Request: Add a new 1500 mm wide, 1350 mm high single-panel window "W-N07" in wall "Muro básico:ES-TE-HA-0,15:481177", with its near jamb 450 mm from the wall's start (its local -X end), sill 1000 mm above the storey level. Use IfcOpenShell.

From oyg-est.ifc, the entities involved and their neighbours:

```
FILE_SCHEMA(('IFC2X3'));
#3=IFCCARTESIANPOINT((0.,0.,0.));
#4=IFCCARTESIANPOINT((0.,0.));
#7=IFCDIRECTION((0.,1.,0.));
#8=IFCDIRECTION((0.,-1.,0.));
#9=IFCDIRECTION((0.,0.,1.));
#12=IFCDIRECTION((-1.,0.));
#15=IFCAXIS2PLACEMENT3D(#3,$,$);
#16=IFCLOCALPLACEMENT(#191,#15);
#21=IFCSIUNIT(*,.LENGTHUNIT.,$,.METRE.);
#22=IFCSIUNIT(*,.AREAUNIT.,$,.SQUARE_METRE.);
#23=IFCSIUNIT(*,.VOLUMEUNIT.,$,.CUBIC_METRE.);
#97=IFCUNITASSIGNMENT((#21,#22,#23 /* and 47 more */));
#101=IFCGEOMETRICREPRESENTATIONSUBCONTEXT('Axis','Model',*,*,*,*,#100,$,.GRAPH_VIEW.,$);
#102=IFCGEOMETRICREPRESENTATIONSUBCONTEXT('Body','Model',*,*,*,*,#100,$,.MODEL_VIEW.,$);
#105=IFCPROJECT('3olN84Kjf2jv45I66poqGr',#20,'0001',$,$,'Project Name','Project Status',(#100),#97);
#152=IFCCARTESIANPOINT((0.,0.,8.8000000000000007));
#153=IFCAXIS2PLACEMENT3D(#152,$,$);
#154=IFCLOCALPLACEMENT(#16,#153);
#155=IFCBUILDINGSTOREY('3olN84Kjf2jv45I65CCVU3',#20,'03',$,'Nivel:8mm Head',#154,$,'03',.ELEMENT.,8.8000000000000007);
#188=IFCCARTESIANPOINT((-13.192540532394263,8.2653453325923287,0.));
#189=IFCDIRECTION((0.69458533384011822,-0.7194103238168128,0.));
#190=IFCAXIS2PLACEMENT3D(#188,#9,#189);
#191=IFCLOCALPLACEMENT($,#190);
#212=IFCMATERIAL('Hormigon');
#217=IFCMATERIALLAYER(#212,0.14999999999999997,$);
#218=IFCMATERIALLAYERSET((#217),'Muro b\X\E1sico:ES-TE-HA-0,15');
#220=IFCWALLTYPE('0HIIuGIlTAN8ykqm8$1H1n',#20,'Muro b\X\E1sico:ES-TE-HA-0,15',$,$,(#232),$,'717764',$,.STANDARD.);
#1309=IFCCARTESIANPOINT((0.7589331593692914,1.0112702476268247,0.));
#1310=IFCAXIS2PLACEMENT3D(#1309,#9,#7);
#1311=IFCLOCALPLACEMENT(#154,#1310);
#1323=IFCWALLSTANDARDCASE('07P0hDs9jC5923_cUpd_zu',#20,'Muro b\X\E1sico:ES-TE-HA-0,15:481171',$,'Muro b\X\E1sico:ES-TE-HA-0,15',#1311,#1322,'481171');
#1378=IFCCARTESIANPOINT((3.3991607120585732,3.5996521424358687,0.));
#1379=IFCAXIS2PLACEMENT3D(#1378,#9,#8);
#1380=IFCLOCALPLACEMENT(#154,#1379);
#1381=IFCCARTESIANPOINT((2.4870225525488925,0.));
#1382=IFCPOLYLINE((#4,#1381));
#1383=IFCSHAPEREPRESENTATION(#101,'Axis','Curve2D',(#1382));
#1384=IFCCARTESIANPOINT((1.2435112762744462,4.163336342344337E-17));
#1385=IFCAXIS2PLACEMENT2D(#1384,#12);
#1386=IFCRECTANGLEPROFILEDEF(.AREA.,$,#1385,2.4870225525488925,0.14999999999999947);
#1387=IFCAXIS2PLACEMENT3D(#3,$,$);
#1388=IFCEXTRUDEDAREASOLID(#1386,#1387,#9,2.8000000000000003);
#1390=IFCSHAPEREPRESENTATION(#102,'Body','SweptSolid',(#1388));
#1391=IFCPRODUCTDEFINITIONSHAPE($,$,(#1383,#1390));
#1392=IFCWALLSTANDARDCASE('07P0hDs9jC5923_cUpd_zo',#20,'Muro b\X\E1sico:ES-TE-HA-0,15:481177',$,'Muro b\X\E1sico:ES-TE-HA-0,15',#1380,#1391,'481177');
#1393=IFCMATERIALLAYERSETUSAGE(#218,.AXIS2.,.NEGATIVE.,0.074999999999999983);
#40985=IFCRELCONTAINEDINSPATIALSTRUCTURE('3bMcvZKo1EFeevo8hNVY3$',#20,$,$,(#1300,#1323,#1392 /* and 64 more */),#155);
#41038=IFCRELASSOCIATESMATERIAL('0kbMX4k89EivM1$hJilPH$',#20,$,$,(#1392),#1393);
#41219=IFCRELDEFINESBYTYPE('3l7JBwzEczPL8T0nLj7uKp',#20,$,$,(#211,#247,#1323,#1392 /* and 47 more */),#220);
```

```python
import numpy as np
import ifcopenshell
import ifcopenshell.api.feature
import ifcopenshell.api.geometry
import ifcopenshell.api.root
import ifcopenshell.api.spatial
import ifcopenshell.api.type
import ifcopenshell.geom
import ifcopenshell.util.element
import ifcopenshell.util.placement
import ifcopenshell.util.representation
import ifcopenshell.util.shape
import ifcopenshell.util.unit

model = ifcopenshell.open("oyg-est.ifc")
unit_scale = ifcopenshell.util.unit.calculate_unit_scale(model)
settings = ifcopenshell.geom.settings()


def volume(element):
    """Net volume in cubic metres, openings subtracted."""
    shape = ifcopenshell.geom.create_shape(settings, element)
    return ifcopenshell.util.shape.get_volume(shape.geometry)


wall = model.by_id(1392)
storey = ifcopenshell.util.element.get_container(wall, ifc_class="IfcBuildingStorey")
context = ifcopenshell.util.representation.get_context(model, "Model", "Body", "MODEL_VIEW")
before = volume(wall)

width, height, from_end, sill = 1.5, 1.35, 0.45, 1  # metres

# The wall runs along its own X axis, and the end named is its -X end.
wall_shape = ifcopenshell.geom.create_shape(settings, wall)
x, y, z = ifcopenshell.util.shape.get_vertices(wall_shape.geometry).T
start = x.min() + from_end
face, thickness = float(y.min()), float(y.max() - y.min())
wall_matrix = ifcopenshell.util.placement.get_local_placement(wall.ObjectPlacement)
level = ifcopenshell.util.placement.get_local_placement(storey.ObjectPlacement)[2, 3]


def in_wall(x, y):
    """Placement at x, y metres in the wall's axes, at sill height."""
    matrix = wall_matrix.copy()
    matrix[:, 3] = wall_matrix @ np.array([x / unit_scale, y / unit_scale, 0.0, 1.0])
    matrix[2, 3] = level + sill / unit_scale
    return matrix


# Opening: a box that overshoots both wall faces by 50 mm.
opening = ifcopenshell.api.root.create_entity(model, ifc_class="IfcOpeningElement")
box = ifcopenshell.api.geometry.add_wall_representation(
    model, context=context, length=width, height=height, thickness=thickness + 0.1
)
ifcopenshell.api.geometry.assign_representation(model, product=opening, representation=box)
ifcopenshell.api.geometry.edit_object_placement(model, product=opening, matrix=in_wall(start, face - 0.05), is_si=False)
ifcopenshell.api.feature.add_feature(model, feature=opening, element=wall)

window = ifcopenshell.api.root.create_entity(model, ifc_class="IfcWindow", name="W-N07")
window.OverallWidth, window.OverallHeight = width / unit_scale, height / unit_scale
body = ifcopenshell.api.geometry.add_window_representation(
    model,
    context=context,
    overall_width=window.OverallWidth,
    overall_height=window.OverallHeight,
    partition_type="SINGLE_PANEL",
)
ifcopenshell.api.geometry.assign_representation(model, product=window, representation=body)
ifcopenshell.api.spatial.assign_container(model, products=[window], relating_structure=storey)
fills = ifcopenshell.api.feature.add_filling(model, opening=opening, element=window)
fills.OwnerHistory = window.OwnerHistory  # required in IFC2X3

# IFC2X3 keeps the operation on the window style.
style = ifcopenshell.api.root.create_entity(model, ifc_class="IfcWindowStyle", name="W-N07")
style.OperationType, style.ConstructionType = "SINGLE_PANEL", "NOTDEFINED"
style.ParameterTakesPrecedence = style.Sizeable = False
ifcopenshell.api.type.assign_type(model, related_objects=[window], relating_type=style)

# Centre the window in the wall's thickness.
ifcopenshell.api.geometry.edit_object_placement(model, product=window, matrix=in_wall(start, face), is_si=False)
window_shape = ifcopenshell.geom.create_shape(settings, window)
depth = ifcopenshell.util.shape.get_vertices(window_shape.geometry)[:, 1]
offset = face + thickness / 2 - (depth.min() + depth.max()) / 2
ifcopenshell.api.geometry.edit_object_placement(model, product=window, matrix=in_wall(start, offset), is_si=False)

after = volume(wall)

print(f"wall volume {before:.3f} -> {after:.3f} m3")

model.write("oyg-est_rev.ifc")
```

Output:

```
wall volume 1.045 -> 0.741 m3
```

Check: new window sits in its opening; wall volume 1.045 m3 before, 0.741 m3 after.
